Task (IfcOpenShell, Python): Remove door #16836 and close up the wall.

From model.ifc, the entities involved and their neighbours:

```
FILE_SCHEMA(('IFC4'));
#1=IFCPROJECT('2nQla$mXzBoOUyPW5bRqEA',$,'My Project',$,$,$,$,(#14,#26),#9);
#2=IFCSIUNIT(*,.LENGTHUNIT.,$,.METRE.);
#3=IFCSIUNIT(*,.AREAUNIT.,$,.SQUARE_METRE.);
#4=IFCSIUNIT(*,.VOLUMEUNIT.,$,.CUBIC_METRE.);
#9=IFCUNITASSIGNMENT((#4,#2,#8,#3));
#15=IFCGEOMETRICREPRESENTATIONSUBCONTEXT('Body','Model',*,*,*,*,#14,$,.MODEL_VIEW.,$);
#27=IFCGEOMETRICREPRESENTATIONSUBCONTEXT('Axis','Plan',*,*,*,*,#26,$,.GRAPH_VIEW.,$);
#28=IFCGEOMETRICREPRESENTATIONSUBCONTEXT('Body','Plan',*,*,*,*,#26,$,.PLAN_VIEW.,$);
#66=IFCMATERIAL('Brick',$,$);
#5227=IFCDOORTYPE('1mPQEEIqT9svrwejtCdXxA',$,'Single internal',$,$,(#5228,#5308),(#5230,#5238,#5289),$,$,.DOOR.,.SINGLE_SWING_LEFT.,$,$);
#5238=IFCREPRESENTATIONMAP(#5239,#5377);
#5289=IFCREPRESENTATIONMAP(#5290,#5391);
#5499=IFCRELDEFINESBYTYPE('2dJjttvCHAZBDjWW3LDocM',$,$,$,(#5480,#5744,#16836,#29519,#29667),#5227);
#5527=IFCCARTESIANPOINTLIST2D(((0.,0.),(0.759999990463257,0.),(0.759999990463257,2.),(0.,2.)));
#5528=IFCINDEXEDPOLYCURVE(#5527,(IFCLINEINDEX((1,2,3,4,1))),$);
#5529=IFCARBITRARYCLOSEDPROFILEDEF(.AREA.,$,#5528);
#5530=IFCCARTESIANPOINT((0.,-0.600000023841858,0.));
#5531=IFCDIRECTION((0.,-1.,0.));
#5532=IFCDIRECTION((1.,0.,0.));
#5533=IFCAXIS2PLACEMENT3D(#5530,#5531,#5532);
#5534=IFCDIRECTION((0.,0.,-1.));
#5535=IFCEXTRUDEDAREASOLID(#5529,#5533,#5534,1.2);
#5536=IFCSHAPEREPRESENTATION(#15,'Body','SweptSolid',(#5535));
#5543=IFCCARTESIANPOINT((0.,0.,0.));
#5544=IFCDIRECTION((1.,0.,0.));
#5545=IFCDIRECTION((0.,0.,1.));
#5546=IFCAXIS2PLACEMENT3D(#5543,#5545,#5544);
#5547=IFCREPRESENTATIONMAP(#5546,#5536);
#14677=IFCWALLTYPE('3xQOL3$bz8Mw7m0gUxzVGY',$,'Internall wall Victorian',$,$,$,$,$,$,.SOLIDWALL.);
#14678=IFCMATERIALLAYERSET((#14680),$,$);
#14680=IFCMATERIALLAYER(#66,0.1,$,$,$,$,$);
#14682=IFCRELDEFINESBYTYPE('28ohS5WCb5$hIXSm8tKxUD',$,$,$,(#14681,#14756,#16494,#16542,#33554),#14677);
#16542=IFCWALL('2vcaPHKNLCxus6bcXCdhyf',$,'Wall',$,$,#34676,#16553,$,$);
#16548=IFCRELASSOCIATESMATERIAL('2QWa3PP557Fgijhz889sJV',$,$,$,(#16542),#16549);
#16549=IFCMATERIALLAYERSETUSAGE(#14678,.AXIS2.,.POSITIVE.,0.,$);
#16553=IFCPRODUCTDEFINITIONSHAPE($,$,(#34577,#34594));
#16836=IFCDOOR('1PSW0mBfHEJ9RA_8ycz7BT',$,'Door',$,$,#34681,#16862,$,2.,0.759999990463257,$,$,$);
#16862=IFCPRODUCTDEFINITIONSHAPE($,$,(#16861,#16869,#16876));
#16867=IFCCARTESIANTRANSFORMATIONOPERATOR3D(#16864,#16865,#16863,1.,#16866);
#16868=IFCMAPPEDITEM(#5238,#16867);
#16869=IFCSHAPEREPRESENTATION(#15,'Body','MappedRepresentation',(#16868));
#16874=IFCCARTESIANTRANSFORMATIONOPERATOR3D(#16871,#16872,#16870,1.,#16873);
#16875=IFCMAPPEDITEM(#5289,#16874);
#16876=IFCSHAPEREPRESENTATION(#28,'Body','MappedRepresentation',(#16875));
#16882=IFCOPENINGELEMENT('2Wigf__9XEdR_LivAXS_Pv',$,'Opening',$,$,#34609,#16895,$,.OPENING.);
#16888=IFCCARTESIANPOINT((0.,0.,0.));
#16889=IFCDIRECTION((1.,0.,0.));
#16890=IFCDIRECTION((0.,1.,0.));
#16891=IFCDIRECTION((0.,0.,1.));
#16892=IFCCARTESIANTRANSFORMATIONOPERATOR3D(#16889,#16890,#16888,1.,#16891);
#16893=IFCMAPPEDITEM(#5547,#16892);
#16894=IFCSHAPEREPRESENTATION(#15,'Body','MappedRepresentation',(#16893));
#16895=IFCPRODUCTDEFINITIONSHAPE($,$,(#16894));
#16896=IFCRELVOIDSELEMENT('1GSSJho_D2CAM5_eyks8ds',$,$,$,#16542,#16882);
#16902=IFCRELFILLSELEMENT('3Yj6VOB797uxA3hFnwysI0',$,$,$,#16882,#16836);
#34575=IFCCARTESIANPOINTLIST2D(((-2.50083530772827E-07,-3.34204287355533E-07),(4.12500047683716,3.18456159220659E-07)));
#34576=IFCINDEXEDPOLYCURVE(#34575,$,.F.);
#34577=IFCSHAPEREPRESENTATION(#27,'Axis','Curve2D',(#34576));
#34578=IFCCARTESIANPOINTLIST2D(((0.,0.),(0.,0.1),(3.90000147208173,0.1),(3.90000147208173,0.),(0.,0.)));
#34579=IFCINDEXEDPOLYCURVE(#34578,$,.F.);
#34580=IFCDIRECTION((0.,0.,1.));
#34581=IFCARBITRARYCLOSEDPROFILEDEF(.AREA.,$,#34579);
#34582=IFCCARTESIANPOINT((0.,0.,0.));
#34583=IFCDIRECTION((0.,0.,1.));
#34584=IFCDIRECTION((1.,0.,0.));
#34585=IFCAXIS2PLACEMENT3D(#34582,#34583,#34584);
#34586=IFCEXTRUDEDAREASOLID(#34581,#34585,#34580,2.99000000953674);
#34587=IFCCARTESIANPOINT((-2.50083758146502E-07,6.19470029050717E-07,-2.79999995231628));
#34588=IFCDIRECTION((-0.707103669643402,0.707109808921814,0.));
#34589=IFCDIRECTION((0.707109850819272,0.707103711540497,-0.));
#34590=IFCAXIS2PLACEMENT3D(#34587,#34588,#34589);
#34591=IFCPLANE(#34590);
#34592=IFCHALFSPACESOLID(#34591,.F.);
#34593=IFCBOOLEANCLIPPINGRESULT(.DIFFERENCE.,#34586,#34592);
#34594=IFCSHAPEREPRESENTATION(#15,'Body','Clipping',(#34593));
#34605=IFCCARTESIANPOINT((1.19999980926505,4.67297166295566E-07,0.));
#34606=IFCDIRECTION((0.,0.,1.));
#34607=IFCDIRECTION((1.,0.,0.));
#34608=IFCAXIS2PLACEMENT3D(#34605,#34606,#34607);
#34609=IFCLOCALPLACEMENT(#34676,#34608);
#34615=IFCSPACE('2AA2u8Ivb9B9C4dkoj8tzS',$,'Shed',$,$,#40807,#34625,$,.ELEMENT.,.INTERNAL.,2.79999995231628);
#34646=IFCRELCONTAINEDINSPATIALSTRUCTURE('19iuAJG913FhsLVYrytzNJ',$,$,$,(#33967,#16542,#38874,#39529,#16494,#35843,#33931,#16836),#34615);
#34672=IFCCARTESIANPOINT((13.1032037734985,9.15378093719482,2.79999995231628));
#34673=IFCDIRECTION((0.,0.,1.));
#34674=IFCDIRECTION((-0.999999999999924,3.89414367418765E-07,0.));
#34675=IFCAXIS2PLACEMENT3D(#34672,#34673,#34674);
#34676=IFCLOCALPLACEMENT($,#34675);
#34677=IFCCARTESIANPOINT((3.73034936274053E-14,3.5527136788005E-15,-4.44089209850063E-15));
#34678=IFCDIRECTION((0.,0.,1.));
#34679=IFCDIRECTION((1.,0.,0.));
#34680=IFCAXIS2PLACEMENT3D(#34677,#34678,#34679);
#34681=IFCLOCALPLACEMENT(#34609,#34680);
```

```python
import ifcopenshell
import ifcopenshell.api.feature
import ifcopenshell.api.root
import ifcopenshell.geom
import ifcopenshell.util.shape

model = ifcopenshell.open("model.ifc")
settings = ifcopenshell.geom.settings()


def volume(element):
    """Net volume in cubic metres, openings subtracted."""
    shape = ifcopenshell.geom.create_shape(settings, element)
    return ifcopenshell.util.shape.get_volume(shape.geometry)


door = model.by_guid("1PSW0mBfHEJ9RA_8ycz7BT")
opening = door.FillsVoids[0].RelatingOpeningElement
wall = opening.VoidsElements[0].RelatingBuildingElement
before = volume(wall)

ifcopenshell.api.root.remove_product(model, product=door)
ifcopenshell.api.feature.remove_feature(model, feature=opening)

after = volume(wall)

print(f"wall volume {before:.3f} -> {after:.3f} m3")

model.write("model-out.ifc")
```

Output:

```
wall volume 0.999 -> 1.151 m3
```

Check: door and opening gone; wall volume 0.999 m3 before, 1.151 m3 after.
